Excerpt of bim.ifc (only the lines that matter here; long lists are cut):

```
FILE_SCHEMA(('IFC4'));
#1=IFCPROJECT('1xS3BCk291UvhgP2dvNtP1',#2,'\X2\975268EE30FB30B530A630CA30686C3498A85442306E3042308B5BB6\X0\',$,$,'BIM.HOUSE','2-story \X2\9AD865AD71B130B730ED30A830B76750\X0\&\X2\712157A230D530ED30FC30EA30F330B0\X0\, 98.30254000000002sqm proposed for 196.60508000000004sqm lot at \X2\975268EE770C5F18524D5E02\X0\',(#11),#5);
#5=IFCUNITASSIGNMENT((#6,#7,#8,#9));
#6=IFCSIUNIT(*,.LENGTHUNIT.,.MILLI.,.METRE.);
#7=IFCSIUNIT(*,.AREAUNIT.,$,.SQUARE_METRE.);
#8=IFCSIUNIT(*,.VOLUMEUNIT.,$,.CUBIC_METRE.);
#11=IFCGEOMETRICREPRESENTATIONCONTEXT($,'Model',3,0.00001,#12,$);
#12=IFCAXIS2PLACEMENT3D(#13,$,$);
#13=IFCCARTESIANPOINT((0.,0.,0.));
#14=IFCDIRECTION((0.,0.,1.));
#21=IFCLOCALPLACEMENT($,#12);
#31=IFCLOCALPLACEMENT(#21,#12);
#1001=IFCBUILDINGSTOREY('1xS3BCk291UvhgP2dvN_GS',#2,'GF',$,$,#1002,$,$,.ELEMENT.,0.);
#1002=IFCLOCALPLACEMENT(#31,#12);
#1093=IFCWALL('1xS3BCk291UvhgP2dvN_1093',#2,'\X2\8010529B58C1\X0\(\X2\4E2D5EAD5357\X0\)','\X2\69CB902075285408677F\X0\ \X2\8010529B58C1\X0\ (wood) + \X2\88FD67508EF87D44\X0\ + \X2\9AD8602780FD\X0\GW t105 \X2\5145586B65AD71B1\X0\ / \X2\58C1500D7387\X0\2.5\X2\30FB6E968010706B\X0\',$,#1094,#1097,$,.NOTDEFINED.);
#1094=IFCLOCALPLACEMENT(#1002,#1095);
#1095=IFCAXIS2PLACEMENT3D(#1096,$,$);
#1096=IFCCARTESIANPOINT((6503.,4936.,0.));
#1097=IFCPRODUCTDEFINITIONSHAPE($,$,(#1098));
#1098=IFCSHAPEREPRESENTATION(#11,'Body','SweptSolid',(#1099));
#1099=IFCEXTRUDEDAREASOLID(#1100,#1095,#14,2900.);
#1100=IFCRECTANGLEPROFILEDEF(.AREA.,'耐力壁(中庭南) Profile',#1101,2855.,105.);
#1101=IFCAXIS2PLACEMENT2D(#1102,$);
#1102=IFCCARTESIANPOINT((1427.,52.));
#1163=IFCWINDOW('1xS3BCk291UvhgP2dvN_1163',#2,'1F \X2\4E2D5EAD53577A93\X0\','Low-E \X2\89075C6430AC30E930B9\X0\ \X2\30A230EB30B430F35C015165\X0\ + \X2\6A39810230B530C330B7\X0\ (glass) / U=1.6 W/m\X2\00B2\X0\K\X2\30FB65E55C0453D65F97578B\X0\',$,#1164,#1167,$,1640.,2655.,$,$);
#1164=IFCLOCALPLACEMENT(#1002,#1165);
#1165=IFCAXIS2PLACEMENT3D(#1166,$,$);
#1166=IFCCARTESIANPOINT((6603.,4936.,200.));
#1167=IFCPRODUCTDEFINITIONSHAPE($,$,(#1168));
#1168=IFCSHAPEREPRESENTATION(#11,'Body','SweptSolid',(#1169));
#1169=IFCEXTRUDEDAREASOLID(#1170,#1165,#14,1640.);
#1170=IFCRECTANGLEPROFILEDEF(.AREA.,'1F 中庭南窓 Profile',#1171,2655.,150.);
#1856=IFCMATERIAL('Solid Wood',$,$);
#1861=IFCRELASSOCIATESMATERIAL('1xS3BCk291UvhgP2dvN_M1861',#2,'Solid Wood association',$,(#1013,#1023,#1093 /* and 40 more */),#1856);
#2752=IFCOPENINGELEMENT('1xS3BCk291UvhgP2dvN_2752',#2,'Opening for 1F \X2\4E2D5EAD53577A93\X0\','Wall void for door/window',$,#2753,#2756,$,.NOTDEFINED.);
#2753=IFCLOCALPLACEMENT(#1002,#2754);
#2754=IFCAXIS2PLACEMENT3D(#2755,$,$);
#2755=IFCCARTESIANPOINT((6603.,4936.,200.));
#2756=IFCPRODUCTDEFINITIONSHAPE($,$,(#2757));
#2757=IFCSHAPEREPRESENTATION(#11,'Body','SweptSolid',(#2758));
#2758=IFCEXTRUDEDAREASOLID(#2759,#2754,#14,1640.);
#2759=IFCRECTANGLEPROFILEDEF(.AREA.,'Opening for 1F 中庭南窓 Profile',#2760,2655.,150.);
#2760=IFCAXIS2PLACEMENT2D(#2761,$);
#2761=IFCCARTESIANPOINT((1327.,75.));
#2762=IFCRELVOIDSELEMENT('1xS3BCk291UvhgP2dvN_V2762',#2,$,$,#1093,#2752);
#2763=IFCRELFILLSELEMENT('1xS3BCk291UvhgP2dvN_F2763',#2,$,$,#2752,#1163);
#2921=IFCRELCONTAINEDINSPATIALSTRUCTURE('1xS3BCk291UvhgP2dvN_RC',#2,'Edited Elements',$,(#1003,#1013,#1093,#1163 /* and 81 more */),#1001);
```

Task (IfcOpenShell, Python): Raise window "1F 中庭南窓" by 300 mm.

```python
import numpy as np
import ifcopenshell
import ifcopenshell.api.geometry
import ifcopenshell.util.placement
import ifcopenshell.util.unit

model = ifcopenshell.open("bim.ifc")
unit_scale = ifcopenshell.util.unit.calculate_unit_scale(model)

window = model.by_guid("1xS3BCk291UvhgP2dvN_1163")
opening = window.FillsVoids[0].RelatingOpeningElement
dz = 0.3 / unit_scale

shift = np.array([0.0, 0.0, dz])
# The window is not placed relative to its opening, so move both.
for product in (opening, window):
    matrix = ifcopenshell.util.placement.get_local_placement(product.ObjectPlacement)
    matrix[:3, 3] += shift
    ifcopenshell.api.geometry.edit_object_placement(model, product=product, matrix=matrix, is_si=False)

print(f"moved by {dz * unit_scale:+.3f} m")

model.write("bim_v2.ifc")
```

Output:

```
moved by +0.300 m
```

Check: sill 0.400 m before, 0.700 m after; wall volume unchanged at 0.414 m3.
